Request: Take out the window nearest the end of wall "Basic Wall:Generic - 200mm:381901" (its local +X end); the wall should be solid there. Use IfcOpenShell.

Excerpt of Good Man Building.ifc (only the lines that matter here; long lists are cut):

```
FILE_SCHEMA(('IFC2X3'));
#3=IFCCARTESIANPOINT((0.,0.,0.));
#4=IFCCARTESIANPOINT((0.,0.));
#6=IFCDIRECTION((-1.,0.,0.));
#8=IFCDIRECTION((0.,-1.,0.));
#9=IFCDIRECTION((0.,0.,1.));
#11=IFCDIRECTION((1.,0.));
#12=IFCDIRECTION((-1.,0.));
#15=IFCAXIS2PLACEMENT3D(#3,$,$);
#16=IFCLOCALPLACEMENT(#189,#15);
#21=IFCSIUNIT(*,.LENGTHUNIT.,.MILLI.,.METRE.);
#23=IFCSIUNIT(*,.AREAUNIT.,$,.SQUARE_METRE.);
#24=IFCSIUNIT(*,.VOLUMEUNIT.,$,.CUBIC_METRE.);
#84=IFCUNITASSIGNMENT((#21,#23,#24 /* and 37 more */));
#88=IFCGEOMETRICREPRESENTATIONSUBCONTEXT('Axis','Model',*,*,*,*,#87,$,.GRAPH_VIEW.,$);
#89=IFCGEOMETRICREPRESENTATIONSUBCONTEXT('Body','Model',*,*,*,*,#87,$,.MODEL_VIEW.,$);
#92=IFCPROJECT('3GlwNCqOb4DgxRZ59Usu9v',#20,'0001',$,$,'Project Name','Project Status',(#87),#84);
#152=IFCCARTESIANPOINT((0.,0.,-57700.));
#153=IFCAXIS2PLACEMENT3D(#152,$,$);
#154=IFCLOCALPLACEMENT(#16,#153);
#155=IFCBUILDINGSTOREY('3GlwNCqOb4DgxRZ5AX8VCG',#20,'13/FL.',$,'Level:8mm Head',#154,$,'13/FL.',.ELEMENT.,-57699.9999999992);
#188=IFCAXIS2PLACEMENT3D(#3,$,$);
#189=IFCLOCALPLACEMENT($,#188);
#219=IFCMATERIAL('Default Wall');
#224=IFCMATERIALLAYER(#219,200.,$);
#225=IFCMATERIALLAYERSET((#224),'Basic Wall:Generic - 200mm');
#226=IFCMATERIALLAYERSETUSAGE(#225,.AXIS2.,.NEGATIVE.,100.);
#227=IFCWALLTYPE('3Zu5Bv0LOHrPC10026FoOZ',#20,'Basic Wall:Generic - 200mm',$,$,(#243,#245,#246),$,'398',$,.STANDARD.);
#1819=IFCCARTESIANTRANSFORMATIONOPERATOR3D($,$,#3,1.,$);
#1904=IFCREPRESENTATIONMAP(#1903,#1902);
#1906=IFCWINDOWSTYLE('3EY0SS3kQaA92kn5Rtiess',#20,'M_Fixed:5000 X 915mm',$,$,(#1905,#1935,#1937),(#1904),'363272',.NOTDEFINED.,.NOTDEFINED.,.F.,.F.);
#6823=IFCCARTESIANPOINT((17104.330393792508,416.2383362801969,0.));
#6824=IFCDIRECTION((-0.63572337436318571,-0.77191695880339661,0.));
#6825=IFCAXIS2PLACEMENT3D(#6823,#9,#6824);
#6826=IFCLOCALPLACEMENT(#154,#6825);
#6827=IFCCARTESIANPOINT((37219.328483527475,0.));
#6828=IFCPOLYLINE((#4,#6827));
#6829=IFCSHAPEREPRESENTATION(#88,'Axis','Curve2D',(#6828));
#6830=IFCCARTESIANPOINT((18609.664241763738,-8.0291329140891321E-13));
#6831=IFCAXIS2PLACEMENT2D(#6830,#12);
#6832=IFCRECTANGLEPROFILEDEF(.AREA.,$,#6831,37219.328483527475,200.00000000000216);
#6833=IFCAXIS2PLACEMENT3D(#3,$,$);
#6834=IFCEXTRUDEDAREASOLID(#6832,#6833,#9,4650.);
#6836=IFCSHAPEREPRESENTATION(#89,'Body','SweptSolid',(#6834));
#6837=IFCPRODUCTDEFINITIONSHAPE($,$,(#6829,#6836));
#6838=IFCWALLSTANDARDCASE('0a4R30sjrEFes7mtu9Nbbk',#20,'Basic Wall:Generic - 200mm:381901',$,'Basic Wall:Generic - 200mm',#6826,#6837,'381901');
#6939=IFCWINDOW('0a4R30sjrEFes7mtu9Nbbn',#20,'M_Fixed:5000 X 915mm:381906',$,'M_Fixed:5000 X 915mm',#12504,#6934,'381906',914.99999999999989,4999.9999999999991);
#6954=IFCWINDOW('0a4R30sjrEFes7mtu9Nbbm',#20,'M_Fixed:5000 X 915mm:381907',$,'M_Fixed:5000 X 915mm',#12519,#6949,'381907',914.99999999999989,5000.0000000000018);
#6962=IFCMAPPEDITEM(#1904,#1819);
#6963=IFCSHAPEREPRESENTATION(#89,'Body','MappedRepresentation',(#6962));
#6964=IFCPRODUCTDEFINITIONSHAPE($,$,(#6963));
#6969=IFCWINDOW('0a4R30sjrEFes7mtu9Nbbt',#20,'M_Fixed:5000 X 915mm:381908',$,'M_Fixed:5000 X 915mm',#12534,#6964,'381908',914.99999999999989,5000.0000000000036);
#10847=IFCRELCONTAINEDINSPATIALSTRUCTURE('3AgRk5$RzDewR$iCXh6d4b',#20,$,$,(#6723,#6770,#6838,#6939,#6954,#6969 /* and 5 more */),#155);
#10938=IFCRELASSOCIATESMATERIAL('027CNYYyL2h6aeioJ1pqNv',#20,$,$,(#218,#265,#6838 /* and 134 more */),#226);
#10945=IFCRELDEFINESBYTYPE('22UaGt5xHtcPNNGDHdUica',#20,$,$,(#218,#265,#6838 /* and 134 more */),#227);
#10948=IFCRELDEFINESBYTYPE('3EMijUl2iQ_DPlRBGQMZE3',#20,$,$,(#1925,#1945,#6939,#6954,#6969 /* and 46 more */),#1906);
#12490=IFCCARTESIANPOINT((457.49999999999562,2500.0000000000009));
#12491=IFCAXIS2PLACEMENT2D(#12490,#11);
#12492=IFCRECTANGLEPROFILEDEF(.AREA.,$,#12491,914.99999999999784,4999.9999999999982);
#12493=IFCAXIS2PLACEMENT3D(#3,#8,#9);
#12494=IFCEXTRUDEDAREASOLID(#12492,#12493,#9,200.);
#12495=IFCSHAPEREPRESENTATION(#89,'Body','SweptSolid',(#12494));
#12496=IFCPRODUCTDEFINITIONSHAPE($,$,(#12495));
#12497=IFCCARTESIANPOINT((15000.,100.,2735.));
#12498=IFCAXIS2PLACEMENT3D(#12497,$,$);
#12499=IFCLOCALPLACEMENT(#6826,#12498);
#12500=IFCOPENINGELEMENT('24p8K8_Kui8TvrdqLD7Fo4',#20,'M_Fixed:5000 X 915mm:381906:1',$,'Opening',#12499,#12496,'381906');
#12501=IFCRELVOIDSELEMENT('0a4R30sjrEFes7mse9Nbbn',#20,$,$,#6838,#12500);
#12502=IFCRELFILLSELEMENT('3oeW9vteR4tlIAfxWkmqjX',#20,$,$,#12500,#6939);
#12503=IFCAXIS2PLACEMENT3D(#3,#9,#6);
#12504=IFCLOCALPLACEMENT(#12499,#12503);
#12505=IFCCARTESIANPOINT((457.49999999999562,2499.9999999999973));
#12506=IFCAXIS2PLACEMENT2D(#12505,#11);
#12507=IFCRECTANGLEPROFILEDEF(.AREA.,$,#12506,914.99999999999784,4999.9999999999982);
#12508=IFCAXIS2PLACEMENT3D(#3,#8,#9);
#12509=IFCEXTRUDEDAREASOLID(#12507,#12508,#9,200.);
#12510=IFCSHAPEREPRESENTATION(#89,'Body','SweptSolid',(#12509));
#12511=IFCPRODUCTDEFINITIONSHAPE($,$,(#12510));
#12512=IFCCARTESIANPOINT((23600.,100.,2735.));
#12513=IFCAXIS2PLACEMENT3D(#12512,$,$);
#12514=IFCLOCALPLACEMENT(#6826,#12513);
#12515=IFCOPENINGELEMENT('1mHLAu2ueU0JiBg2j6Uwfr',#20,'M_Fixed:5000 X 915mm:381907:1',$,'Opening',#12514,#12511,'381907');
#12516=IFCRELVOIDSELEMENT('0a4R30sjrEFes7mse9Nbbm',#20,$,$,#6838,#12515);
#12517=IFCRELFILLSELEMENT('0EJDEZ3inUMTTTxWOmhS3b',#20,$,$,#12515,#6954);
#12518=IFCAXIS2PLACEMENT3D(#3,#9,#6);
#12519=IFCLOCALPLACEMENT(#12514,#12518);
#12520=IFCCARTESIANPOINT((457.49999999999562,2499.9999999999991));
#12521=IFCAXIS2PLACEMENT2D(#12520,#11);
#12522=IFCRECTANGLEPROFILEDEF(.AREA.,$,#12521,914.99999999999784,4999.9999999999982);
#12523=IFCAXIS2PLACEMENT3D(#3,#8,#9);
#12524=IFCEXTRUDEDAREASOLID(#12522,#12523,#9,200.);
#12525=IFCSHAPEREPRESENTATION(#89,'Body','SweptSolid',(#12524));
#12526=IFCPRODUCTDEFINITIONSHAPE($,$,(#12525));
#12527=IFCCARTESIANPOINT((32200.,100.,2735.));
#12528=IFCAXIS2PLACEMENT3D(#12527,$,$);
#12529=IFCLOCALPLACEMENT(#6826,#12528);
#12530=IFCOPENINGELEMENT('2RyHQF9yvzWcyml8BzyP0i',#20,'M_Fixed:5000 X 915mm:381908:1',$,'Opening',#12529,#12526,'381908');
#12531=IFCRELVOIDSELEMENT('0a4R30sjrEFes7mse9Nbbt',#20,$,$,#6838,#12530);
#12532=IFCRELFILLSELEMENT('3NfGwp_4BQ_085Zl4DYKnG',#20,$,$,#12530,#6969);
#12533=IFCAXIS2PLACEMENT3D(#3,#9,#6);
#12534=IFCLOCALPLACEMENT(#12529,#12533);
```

```python
import ifcopenshell
import ifcopenshell.api.feature
import ifcopenshell.api.root
import ifcopenshell.geom
import ifcopenshell.util.shape

model = ifcopenshell.open("Good Man Building.ifc")
settings = ifcopenshell.geom.settings()


def volume(element):
    """Net volume in cubic metres, openings subtracted."""
    shape = ifcopenshell.geom.create_shape(settings, element)
    return ifcopenshell.util.shape.get_volume(shape.geometry)


window = model.by_guid("0a4R30sjrEFes7mtu9Nbbt")
opening = window.FillsVoids[0].RelatingOpeningElement
wall = opening.VoidsElements[0].RelatingBuildingElement
before = volume(wall)

ifcopenshell.api.root.remove_product(model, product=window)
ifcopenshell.api.feature.remove_feature(model, feature=opening)

after = volume(wall)

print(f"wall volume {before:.3f} -> {after:.3f} m3")

model.write("Good Man Building_edited.ifc")
```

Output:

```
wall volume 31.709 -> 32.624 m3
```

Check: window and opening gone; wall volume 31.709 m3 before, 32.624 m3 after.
